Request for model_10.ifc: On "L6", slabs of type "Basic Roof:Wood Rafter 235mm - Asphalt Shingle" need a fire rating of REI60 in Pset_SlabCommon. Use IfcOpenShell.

First a look at what the model holds.

```python
import ifcopenshell
import ifcopenshell.util.element

model = ifcopenshell.open("model_10.ifc")
print(model.schema)
storey = next(s for s in model.by_type("IfcBuildingStorey") if s.Name == "L6")
slabs = [e for e in ifcopenshell.util.element.get_decomposition(storey) if e.is_a("IfcSlab")]
seen = {}
for e in slabs:
    element_type = ifcopenshell.util.element.get_type(e)
    key = (element_type.Name if element_type != e and element_type else None, ifcopenshell.util.element.get_pset(e, "Pset_SlabCommon", "FireRating"))
    seen[key] = seen.get(key, 0) + 1
for (name, value), count in sorted(seen.items(), key=str):
    print(count, "x", name, "|", value)
```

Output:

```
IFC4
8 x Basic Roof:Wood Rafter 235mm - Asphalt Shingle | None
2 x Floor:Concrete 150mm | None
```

```python
import ifcopenshell
import ifcopenshell.api.pset
import ifcopenshell.util.element

model = ifcopenshell.open("model_10.ifc")

storey = next(s for s in model.by_type("IfcBuildingStorey") if s.Name == "L6")
slabs = [e for e in ifcopenshell.util.element.get_decomposition(storey) if e.is_a("IfcSlab")]

count = 0
for e in slabs:
    element_type = ifcopenshell.util.element.get_type(e)
    if element_type in (None, e) or element_type.Name != "Basic Roof:Wood Rafter 235mm - Asphalt Shingle":
        continue
    # add_pset returns the element's existing set when there is one.
    pset = ifcopenshell.api.pset.add_pset(model, product=e, name="Pset_SlabCommon")
    ifcopenshell.api.pset.edit_pset(model, pset=pset, properties={"FireRating": "REI60"})
    count += 1

print(count, "slabs updated")

model.write("model_10_v2.ifc")
```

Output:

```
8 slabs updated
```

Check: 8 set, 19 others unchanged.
